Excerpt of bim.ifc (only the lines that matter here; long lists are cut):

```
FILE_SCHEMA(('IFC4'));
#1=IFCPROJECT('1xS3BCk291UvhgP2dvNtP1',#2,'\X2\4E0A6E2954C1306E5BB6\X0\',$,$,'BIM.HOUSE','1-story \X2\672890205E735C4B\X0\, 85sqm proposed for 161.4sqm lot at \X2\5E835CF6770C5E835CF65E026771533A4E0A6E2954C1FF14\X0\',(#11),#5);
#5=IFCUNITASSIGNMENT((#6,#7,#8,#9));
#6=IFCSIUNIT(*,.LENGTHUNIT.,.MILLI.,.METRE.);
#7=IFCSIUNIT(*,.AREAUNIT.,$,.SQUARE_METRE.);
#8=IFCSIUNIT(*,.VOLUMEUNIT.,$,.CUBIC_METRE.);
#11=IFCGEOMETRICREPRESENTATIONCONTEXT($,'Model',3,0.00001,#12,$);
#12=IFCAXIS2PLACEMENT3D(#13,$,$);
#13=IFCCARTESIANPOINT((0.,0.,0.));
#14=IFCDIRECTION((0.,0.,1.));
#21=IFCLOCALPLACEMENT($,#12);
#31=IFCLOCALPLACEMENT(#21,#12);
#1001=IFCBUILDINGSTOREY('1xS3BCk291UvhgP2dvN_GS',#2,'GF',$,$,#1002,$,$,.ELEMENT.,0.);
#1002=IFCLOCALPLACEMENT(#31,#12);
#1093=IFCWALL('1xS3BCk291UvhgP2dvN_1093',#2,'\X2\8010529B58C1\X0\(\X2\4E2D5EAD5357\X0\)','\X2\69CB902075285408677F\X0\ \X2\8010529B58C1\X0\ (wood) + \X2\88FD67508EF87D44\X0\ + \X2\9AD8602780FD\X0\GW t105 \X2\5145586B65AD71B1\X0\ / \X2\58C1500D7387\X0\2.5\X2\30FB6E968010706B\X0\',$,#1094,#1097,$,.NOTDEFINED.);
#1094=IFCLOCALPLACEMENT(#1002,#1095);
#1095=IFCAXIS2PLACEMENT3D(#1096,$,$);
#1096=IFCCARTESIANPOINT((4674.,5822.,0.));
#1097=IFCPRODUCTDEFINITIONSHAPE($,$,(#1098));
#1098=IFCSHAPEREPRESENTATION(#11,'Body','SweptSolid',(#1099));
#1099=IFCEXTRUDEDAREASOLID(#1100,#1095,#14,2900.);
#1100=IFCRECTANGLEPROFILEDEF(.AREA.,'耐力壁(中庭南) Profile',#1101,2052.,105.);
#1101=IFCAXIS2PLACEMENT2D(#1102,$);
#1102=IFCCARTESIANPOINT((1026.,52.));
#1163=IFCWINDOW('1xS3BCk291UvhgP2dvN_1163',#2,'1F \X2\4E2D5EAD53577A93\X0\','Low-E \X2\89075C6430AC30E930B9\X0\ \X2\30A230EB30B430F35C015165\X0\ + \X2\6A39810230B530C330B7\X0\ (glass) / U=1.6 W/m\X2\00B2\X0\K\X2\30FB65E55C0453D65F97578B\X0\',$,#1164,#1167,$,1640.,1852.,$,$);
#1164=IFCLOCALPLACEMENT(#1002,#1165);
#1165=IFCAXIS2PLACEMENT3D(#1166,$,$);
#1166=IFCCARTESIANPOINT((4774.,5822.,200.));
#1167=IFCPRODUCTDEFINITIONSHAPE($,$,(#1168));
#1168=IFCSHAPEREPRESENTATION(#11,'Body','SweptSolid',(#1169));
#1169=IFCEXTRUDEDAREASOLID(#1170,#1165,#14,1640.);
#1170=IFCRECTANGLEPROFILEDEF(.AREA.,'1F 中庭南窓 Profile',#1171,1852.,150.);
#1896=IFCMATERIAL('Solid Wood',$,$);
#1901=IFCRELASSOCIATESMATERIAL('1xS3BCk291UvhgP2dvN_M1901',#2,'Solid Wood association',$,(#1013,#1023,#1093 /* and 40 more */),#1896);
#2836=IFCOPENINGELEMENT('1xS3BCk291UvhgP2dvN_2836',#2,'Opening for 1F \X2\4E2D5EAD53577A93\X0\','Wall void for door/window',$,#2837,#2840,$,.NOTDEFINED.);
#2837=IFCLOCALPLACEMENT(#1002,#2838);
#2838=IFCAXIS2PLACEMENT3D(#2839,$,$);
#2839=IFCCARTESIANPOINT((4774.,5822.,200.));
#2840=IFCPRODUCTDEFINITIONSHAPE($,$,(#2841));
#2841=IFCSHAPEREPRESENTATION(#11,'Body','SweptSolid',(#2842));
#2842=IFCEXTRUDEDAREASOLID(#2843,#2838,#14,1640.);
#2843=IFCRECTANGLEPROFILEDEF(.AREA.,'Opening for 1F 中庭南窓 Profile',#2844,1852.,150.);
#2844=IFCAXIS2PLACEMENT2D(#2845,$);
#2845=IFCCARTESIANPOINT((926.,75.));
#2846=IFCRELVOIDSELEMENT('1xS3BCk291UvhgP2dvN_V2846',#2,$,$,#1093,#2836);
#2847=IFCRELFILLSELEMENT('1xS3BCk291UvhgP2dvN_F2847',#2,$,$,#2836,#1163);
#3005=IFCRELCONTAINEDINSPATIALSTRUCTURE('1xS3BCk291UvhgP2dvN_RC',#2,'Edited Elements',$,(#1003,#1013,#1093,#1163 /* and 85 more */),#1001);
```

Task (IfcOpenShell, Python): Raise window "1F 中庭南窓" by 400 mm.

```python
import numpy as np
import ifcopenshell
import ifcopenshell.api.geometry
import ifcopenshell.util.placement
import ifcopenshell.util.unit

model = ifcopenshell.open("bim.ifc")
unit_scale = ifcopenshell.util.unit.calculate_unit_scale(model)

window = model.by_id(1163)
opening = window.FillsVoids[0].RelatingOpeningElement
dz = 400.0

shift = np.array([0.0, 0.0, dz])
# The window is not placed relative to its opening, so move both.
for product in (opening, window):
    matrix = ifcopenshell.util.placement.get_local_placement(product.ObjectPlacement)
    matrix[:3, 3] += shift
    ifcopenshell.api.geometry.edit_object_placement(model, product=product, matrix=matrix, is_si=False)

print(f"moved by {dz * unit_scale:+.3f} m")

model.write("bim_v2.ifc")
```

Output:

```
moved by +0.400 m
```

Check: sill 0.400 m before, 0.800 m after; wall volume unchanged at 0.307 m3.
